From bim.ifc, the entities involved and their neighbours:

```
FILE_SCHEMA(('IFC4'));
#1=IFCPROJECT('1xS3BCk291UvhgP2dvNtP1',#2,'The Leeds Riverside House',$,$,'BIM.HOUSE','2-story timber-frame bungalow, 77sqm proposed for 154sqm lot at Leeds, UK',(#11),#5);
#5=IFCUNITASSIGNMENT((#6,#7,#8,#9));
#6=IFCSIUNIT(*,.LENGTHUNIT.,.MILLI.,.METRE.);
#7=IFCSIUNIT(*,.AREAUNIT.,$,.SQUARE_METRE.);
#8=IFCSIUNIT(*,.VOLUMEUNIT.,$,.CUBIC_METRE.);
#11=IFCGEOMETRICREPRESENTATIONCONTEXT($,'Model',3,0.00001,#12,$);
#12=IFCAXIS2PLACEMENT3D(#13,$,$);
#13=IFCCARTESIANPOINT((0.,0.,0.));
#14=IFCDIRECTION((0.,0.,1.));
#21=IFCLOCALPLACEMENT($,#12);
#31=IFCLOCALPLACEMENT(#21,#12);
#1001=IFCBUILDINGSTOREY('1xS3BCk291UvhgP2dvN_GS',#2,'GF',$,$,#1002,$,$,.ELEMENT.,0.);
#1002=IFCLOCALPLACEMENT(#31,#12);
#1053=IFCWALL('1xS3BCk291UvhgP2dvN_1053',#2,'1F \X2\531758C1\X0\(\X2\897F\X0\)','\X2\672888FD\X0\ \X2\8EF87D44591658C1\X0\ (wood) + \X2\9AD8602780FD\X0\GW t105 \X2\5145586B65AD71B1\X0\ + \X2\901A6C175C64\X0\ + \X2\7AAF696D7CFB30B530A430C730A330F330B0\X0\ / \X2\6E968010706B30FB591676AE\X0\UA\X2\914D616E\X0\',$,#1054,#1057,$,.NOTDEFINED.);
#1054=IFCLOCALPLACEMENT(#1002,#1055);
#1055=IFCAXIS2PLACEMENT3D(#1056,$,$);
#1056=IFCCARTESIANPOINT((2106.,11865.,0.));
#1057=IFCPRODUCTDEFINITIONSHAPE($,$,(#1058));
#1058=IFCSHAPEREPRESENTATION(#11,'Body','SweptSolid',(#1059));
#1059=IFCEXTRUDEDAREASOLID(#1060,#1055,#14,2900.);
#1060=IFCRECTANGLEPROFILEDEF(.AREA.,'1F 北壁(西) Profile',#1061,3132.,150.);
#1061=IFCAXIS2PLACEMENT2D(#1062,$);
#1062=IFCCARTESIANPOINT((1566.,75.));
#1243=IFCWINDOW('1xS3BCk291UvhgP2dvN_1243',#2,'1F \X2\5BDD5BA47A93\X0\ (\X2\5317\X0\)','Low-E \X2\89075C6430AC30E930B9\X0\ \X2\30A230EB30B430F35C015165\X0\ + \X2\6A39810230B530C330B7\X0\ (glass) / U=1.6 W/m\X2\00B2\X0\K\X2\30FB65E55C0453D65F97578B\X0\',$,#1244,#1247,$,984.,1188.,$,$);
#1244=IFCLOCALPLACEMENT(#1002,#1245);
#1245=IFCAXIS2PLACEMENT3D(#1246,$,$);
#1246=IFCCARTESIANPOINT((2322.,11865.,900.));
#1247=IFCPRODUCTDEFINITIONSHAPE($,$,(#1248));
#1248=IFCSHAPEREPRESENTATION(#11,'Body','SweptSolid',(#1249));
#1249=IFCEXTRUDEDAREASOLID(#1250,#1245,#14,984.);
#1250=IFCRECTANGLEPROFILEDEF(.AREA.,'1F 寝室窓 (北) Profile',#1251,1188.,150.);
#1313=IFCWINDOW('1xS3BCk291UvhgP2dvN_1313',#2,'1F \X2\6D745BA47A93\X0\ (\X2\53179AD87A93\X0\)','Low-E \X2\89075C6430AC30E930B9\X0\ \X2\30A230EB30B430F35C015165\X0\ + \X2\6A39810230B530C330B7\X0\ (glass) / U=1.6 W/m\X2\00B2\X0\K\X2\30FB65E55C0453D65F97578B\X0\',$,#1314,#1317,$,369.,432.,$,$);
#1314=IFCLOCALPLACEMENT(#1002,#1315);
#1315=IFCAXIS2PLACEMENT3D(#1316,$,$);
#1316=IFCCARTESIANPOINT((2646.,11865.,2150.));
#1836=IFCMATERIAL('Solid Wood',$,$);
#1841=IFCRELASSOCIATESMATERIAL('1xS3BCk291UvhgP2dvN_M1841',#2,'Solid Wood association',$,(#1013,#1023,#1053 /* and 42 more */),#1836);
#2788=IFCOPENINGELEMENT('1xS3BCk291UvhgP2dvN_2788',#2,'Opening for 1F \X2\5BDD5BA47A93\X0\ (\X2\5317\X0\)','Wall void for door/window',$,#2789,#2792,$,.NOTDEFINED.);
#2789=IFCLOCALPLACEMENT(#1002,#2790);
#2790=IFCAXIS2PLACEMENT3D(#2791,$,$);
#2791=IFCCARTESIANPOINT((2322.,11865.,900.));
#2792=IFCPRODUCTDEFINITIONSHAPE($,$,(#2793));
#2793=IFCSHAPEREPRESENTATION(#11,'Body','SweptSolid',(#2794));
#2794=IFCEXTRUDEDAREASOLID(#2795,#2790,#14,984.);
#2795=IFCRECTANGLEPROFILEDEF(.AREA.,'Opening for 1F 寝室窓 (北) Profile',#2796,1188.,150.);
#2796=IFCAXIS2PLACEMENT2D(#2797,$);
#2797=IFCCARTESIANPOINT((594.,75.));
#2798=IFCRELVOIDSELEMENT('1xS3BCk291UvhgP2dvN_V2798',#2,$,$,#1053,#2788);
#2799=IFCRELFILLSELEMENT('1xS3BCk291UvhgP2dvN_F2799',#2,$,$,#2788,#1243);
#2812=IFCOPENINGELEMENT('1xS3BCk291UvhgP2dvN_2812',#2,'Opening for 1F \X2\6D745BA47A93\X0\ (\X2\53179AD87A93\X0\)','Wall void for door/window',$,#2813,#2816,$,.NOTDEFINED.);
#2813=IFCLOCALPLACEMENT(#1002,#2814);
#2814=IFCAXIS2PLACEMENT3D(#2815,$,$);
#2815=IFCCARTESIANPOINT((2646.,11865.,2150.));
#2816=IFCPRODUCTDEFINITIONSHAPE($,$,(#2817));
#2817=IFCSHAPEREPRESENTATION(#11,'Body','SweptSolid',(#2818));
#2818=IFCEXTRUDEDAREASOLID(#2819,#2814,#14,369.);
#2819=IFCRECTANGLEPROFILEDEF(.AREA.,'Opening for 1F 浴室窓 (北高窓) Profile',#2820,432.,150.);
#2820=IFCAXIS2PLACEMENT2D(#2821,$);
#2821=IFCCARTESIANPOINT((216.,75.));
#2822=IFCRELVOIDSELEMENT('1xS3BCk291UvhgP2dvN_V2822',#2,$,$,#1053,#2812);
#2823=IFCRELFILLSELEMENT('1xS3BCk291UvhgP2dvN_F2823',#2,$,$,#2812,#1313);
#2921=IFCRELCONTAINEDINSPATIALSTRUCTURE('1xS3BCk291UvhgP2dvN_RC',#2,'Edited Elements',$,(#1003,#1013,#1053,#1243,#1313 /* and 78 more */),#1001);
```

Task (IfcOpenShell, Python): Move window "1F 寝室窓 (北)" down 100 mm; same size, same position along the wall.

```python
import numpy as np
import ifcopenshell
import ifcopenshell.api.geometry
import ifcopenshell.util.placement
import ifcopenshell.util.unit

model = ifcopenshell.open("bim.ifc")
unit_scale = ifcopenshell.util.unit.calculate_unit_scale(model)

window = model.by_id(1243)
opening = window.FillsVoids[0].RelatingOpeningElement
dz = -100.0

shift = np.array([0.0, 0.0, dz])
# The window is not placed relative to its opening, so move both.
for product in (opening, window):
    matrix = ifcopenshell.util.placement.get_local_placement(product.ObjectPlacement)
    matrix[:3, 3] += shift
    ifcopenshell.api.geometry.edit_object_placement(model, product=product, matrix=matrix, is_si=False)

print(f"moved by {dz * unit_scale:+.3f} m")

model.write("bim_edited.ifc")
```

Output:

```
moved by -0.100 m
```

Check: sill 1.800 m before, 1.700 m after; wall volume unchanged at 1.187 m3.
